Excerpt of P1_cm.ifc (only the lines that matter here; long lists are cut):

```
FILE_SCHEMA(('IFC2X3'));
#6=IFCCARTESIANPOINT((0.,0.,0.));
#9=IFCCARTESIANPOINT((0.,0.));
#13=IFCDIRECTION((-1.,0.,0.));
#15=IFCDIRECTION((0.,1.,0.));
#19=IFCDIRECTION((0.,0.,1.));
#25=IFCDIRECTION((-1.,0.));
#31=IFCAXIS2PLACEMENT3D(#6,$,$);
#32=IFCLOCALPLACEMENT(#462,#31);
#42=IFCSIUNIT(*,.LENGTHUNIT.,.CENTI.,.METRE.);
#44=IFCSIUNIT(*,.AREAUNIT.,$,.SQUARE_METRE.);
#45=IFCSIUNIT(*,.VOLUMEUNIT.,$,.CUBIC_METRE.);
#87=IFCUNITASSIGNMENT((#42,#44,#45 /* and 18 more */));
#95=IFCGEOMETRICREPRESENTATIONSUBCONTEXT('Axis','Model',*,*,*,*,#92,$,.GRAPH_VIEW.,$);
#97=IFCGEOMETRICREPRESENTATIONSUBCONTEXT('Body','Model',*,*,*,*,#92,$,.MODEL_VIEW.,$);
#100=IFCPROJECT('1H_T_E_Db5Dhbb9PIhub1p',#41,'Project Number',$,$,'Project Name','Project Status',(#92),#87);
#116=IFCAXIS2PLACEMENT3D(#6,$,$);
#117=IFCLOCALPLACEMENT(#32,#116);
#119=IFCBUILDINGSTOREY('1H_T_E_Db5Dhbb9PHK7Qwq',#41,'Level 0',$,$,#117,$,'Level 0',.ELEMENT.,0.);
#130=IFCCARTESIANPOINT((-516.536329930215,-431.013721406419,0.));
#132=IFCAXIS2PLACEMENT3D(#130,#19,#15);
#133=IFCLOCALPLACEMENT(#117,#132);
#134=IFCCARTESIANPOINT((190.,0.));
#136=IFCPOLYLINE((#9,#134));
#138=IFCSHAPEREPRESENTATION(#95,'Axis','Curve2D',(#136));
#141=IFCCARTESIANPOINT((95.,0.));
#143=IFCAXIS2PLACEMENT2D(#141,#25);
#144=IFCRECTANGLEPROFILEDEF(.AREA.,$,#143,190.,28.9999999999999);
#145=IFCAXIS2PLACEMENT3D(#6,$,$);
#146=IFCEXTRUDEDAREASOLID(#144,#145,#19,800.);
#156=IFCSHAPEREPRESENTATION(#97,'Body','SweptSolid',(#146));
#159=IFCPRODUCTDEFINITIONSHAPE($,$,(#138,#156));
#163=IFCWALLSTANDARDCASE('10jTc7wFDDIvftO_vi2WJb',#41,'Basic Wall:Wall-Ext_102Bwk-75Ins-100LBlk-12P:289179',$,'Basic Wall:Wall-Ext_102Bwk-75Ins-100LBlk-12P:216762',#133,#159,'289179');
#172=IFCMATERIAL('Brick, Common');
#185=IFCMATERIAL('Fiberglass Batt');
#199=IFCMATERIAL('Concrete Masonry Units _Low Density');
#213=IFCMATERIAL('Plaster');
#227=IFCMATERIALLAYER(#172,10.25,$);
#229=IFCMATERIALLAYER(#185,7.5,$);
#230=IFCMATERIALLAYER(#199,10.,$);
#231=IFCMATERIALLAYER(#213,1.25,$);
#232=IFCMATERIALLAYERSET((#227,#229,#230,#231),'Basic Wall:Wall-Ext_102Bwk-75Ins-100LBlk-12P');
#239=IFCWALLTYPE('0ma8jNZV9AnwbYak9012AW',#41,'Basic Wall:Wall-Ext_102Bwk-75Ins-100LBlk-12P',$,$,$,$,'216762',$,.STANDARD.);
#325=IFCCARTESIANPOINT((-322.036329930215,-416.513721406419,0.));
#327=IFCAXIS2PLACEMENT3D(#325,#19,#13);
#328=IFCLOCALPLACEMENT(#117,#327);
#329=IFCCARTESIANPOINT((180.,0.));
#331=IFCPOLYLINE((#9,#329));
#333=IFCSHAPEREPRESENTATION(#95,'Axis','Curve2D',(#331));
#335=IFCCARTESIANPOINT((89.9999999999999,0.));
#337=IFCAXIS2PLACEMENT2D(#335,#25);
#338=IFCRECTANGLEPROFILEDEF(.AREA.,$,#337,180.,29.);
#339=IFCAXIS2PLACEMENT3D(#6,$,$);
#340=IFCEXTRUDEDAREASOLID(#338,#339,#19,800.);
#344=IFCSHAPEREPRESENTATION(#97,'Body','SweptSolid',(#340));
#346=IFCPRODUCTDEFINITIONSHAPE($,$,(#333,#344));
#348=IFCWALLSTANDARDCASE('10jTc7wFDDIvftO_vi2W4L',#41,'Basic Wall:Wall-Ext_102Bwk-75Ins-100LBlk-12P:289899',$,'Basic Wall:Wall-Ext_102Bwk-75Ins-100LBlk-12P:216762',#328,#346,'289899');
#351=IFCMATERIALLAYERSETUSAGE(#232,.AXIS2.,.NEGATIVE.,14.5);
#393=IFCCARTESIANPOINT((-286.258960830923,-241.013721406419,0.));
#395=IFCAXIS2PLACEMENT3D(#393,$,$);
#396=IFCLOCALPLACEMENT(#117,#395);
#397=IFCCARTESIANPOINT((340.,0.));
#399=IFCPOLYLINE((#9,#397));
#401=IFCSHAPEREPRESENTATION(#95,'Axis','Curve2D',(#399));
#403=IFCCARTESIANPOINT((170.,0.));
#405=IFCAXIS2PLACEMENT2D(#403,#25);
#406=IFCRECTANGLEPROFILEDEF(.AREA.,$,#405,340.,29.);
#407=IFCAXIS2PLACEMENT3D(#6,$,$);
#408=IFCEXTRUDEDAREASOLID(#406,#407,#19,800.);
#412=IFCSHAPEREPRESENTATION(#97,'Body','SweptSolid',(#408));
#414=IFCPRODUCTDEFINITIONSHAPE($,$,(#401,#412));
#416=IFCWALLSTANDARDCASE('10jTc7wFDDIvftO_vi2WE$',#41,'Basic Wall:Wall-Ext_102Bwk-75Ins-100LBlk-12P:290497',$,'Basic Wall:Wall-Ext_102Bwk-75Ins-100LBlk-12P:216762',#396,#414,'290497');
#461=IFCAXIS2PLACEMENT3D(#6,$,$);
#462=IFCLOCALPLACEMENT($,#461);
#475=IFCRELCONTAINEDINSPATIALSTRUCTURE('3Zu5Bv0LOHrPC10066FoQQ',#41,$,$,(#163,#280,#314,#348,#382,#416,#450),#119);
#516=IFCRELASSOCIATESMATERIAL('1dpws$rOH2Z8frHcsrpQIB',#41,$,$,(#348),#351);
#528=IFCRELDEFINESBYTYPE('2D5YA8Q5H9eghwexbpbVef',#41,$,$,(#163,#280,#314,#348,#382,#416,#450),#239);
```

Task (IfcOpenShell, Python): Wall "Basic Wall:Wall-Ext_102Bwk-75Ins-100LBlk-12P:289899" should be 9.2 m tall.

```python
import ifcopenshell
import ifcopenshell.geom
import ifcopenshell.util.representation
import ifcopenshell.util.shape
import ifcopenshell.util.unit

model = ifcopenshell.open("P1_cm.ifc")
unit_scale = ifcopenshell.util.unit.calculate_unit_scale(model)
settings = ifcopenshell.geom.settings()


def volume(element):
    """Net volume in cubic metres, openings subtracted."""
    shape = ifcopenshell.geom.create_shape(settings, element)
    return ifcopenshell.util.shape.get_volume(shape.geometry)


wall = model.by_id(348)
before = volume(wall)

body = ifcopenshell.util.representation.get_representation(wall, "Model", "Body")
solid = body.Items[0]
old_height = solid.Depth
solid.Depth = 9.2 / unit_scale
after = volume(wall)

print(f"height {old_height:g} -> {solid.Depth:g}, volume {before:.3f} -> {after:.3f} m3")

model.write("P1_cm_edited.ifc")
```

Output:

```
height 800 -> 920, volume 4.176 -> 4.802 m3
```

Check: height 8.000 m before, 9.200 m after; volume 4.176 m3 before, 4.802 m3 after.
